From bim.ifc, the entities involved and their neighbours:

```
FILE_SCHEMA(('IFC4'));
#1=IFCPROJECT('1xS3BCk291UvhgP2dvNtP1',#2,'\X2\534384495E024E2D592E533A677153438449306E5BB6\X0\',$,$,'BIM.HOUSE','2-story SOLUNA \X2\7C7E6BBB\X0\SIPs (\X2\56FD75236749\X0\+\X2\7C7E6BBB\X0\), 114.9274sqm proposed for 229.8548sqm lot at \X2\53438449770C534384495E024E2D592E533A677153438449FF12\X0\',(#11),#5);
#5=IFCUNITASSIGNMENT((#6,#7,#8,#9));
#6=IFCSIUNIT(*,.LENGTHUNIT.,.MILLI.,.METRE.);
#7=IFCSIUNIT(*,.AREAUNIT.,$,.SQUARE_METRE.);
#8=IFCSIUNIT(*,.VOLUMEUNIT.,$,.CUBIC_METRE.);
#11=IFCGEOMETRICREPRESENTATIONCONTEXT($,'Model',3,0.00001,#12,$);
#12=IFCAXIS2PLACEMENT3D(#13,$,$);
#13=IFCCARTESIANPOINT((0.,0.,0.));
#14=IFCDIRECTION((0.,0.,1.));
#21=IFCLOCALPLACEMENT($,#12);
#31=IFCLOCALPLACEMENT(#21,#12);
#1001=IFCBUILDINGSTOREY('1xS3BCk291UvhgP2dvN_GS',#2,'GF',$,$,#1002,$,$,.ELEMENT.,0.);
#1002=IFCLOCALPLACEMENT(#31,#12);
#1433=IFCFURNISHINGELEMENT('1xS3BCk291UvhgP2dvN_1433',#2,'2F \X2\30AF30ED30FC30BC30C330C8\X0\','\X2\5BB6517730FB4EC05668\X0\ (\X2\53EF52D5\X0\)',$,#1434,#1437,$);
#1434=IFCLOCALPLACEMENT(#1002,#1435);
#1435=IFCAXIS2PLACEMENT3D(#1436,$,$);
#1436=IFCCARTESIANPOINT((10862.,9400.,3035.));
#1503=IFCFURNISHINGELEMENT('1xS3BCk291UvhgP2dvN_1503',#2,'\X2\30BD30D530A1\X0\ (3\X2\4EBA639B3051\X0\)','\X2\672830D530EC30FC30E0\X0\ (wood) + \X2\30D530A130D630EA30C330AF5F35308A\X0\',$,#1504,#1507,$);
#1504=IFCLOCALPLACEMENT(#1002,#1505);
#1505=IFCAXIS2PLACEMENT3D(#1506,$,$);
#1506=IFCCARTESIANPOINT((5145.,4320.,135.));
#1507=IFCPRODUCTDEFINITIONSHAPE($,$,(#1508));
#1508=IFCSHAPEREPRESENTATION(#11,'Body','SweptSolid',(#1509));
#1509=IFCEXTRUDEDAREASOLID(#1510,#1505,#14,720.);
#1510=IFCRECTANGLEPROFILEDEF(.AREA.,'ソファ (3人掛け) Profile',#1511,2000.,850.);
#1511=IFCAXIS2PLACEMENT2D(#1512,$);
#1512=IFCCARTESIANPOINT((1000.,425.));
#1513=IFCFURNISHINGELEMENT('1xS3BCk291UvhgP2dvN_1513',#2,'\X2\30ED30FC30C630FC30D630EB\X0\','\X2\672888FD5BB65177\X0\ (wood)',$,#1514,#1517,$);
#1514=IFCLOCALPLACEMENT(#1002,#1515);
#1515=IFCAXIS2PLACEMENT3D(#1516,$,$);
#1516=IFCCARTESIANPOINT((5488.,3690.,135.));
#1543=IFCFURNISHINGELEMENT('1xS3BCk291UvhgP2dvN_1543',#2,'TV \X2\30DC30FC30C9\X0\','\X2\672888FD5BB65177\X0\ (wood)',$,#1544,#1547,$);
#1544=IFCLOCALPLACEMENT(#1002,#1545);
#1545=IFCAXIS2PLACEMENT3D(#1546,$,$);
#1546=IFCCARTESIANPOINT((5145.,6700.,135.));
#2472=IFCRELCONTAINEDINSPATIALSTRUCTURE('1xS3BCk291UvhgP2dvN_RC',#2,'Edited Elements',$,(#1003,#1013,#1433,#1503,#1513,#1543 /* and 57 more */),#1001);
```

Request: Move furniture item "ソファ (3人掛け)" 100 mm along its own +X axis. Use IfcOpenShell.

```python
import ifcopenshell
import ifcopenshell.api.geometry
import ifcopenshell.util.placement

model = ifcopenshell.open("bim.ifc")

item = model.by_id(1503)
matrix = ifcopenshell.util.placement.get_local_placement(item.ObjectPlacement)
matrix[:3, 3] += matrix[:3, 0] * 100.0
ifcopenshell.api.geometry.edit_object_placement(model, product=item, matrix=matrix, is_si=False)

print(ifcopenshell.util.placement.get_local_placement(item.ObjectPlacement).round(3) + 0.0)

model.write("bim_edited.ifc")
```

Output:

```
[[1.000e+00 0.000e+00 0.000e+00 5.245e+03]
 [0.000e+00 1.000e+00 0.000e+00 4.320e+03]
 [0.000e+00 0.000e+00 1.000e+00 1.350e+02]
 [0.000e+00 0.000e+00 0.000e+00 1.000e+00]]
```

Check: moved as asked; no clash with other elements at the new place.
